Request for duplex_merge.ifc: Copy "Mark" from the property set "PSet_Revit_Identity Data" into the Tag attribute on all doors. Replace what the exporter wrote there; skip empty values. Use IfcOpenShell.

First a look at what the model holds.

```python
import ifcopenshell
import ifcopenshell.util.element

model = ifcopenshell.open("duplex_merge.ifc")
print(model.schema)
doors = model.by_type("IfcDoor")
print(len(doors), "doors")
for e in doors[:8]:
    source = ifcopenshell.util.element.get_pset(e, "PSet_Revit_Identity Data", "Mark")
    target = e.Tag
    print(e.id(), repr(source), repr(target), sep=" | ")
```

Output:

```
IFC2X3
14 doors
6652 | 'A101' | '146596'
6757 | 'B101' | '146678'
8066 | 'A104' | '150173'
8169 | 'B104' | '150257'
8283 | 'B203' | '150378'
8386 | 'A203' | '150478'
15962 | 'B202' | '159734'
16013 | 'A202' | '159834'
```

```python
import ifcopenshell
import ifcopenshell.util.element

model = ifcopenshell.open("duplex_merge.ifc")

count = 0
for e in model.by_type("IfcDoor"):
    value = ifcopenshell.util.element.get_pset(e, "PSet_Revit_Identity Data", "Mark")
    current = e.Tag
    if not value or not value.strip() or current == value:
        continue
    e.Tag = value
    count += 1

print(count, "doors updated")

model.write("duplex_merge_rev.ifc")
```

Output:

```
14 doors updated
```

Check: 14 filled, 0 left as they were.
